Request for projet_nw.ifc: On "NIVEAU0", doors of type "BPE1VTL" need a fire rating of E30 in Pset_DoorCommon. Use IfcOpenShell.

First a look at what the model holds.

```python
import ifcopenshell
import ifcopenshell.util.element

model = ifcopenshell.open("projet_nw.ifc")
print(model.schema)
storey = next(s for s in model.by_type("IfcBuildingStorey") if s.Name == "NIVEAU0")
doors = [e for e in ifcopenshell.util.element.get_decomposition(storey) if e.is_a("IfcDoor")]
seen = {}
for e in doors:
    element_type = ifcopenshell.util.element.get_type(e)
    key = (element_type.Name if element_type != e and element_type else None, ifcopenshell.util.element.get_pset(e, "Pset_DoorCommon", "FireRating"))
    seen[key] = seen.get(key, 0) + 1
for (name, value), count in sorted(seen.items(), key=str):
    print(count, "x", name, "|", value)
```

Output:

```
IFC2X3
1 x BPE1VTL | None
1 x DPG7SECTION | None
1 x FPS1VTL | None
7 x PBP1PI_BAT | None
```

```python
import ifcopenshell
import ifcopenshell.api.pset
import ifcopenshell.util.element

model = ifcopenshell.open("projet_nw.ifc")

storey = next(s for s in model.by_type("IfcBuildingStorey") if s.Name == "NIVEAU0")
doors = [e for e in ifcopenshell.util.element.get_decomposition(storey) if e.is_a("IfcDoor")]

count = 0
for e in doors:
    element_type = ifcopenshell.util.element.get_type(e)
    if element_type in (None, e) or element_type.Name != "BPE1VTL":
        continue
    # add_pset returns the element's existing set when there is one.
    pset = ifcopenshell.api.pset.add_pset(model, product=e, name="Pset_DoorCommon")
    ifcopenshell.api.pset.edit_pset(model, pset=pset, properties={"FireRating": "E30"})
    count += 1

print(count, "doors updated")

model.write("projet_nw_updated.ifc")
```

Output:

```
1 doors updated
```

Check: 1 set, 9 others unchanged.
